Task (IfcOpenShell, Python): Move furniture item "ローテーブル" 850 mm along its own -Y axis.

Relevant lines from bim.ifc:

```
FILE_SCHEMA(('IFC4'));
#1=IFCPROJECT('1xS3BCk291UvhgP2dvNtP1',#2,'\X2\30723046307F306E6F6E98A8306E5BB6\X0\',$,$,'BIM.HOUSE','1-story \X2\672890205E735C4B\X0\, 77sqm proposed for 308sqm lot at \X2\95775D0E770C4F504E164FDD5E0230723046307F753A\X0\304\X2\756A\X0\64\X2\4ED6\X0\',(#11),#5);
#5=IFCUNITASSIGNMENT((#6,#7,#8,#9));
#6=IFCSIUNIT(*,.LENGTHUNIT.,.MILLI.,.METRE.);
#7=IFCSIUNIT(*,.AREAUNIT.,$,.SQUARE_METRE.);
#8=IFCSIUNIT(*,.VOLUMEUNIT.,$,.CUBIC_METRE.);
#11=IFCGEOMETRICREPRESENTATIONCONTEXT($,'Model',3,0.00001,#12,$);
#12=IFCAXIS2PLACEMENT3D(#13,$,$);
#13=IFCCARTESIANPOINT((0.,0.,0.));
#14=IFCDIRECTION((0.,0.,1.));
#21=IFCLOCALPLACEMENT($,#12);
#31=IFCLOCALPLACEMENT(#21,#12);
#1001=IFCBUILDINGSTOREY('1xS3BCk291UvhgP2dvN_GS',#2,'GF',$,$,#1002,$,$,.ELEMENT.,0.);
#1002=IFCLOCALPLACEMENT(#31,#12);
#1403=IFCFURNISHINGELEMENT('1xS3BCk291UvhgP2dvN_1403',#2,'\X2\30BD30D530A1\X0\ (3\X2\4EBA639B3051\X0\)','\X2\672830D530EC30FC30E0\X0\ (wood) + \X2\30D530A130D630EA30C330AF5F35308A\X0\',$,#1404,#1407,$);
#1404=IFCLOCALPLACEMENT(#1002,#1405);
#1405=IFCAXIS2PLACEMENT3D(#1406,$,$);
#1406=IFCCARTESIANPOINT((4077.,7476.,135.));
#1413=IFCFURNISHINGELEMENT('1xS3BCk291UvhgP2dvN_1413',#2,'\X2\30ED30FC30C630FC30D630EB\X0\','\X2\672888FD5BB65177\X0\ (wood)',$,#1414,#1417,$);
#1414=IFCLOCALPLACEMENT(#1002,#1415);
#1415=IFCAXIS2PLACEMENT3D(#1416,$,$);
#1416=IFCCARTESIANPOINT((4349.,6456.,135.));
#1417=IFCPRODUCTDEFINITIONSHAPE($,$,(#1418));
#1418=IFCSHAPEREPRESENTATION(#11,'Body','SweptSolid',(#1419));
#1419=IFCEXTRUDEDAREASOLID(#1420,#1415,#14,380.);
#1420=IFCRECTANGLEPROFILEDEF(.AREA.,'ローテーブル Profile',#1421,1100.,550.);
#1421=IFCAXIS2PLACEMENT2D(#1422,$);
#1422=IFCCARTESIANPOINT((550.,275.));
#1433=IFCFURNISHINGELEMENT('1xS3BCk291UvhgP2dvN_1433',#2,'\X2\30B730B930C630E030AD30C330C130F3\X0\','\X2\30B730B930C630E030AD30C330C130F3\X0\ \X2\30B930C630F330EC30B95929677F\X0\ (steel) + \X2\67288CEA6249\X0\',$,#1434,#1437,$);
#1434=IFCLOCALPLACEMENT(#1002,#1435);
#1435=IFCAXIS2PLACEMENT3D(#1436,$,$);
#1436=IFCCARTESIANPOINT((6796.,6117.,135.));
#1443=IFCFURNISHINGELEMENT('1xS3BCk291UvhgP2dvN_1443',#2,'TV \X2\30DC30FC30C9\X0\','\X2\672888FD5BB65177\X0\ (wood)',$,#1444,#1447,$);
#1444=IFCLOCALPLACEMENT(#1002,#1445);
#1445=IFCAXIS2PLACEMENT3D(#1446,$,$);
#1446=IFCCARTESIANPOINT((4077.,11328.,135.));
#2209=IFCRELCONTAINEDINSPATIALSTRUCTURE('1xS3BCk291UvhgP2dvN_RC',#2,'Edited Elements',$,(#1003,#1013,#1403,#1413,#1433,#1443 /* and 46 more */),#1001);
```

```python
import ifcopenshell
import ifcopenshell.api.geometry
import ifcopenshell.util.placement
import ifcopenshell.util.unit

model = ifcopenshell.open("bim.ifc")
unit_scale = ifcopenshell.util.unit.calculate_unit_scale(model)

item = model.by_guid("1xS3BCk291UvhgP2dvN_1413")
matrix = ifcopenshell.util.placement.get_local_placement(item.ObjectPlacement)
matrix[:3, 3] -= matrix[:3, 1] * 0.85 / unit_scale
ifcopenshell.api.geometry.edit_object_placement(model, product=item, matrix=matrix, is_si=False)

print(ifcopenshell.util.placement.get_local_placement(item.ObjectPlacement).round(3) + 0.0)

model.write("bim_edited.ifc")
```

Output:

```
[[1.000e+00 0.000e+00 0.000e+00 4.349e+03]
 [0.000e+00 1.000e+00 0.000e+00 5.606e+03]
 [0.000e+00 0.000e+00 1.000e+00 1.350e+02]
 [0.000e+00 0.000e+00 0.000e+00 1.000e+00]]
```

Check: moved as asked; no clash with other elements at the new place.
